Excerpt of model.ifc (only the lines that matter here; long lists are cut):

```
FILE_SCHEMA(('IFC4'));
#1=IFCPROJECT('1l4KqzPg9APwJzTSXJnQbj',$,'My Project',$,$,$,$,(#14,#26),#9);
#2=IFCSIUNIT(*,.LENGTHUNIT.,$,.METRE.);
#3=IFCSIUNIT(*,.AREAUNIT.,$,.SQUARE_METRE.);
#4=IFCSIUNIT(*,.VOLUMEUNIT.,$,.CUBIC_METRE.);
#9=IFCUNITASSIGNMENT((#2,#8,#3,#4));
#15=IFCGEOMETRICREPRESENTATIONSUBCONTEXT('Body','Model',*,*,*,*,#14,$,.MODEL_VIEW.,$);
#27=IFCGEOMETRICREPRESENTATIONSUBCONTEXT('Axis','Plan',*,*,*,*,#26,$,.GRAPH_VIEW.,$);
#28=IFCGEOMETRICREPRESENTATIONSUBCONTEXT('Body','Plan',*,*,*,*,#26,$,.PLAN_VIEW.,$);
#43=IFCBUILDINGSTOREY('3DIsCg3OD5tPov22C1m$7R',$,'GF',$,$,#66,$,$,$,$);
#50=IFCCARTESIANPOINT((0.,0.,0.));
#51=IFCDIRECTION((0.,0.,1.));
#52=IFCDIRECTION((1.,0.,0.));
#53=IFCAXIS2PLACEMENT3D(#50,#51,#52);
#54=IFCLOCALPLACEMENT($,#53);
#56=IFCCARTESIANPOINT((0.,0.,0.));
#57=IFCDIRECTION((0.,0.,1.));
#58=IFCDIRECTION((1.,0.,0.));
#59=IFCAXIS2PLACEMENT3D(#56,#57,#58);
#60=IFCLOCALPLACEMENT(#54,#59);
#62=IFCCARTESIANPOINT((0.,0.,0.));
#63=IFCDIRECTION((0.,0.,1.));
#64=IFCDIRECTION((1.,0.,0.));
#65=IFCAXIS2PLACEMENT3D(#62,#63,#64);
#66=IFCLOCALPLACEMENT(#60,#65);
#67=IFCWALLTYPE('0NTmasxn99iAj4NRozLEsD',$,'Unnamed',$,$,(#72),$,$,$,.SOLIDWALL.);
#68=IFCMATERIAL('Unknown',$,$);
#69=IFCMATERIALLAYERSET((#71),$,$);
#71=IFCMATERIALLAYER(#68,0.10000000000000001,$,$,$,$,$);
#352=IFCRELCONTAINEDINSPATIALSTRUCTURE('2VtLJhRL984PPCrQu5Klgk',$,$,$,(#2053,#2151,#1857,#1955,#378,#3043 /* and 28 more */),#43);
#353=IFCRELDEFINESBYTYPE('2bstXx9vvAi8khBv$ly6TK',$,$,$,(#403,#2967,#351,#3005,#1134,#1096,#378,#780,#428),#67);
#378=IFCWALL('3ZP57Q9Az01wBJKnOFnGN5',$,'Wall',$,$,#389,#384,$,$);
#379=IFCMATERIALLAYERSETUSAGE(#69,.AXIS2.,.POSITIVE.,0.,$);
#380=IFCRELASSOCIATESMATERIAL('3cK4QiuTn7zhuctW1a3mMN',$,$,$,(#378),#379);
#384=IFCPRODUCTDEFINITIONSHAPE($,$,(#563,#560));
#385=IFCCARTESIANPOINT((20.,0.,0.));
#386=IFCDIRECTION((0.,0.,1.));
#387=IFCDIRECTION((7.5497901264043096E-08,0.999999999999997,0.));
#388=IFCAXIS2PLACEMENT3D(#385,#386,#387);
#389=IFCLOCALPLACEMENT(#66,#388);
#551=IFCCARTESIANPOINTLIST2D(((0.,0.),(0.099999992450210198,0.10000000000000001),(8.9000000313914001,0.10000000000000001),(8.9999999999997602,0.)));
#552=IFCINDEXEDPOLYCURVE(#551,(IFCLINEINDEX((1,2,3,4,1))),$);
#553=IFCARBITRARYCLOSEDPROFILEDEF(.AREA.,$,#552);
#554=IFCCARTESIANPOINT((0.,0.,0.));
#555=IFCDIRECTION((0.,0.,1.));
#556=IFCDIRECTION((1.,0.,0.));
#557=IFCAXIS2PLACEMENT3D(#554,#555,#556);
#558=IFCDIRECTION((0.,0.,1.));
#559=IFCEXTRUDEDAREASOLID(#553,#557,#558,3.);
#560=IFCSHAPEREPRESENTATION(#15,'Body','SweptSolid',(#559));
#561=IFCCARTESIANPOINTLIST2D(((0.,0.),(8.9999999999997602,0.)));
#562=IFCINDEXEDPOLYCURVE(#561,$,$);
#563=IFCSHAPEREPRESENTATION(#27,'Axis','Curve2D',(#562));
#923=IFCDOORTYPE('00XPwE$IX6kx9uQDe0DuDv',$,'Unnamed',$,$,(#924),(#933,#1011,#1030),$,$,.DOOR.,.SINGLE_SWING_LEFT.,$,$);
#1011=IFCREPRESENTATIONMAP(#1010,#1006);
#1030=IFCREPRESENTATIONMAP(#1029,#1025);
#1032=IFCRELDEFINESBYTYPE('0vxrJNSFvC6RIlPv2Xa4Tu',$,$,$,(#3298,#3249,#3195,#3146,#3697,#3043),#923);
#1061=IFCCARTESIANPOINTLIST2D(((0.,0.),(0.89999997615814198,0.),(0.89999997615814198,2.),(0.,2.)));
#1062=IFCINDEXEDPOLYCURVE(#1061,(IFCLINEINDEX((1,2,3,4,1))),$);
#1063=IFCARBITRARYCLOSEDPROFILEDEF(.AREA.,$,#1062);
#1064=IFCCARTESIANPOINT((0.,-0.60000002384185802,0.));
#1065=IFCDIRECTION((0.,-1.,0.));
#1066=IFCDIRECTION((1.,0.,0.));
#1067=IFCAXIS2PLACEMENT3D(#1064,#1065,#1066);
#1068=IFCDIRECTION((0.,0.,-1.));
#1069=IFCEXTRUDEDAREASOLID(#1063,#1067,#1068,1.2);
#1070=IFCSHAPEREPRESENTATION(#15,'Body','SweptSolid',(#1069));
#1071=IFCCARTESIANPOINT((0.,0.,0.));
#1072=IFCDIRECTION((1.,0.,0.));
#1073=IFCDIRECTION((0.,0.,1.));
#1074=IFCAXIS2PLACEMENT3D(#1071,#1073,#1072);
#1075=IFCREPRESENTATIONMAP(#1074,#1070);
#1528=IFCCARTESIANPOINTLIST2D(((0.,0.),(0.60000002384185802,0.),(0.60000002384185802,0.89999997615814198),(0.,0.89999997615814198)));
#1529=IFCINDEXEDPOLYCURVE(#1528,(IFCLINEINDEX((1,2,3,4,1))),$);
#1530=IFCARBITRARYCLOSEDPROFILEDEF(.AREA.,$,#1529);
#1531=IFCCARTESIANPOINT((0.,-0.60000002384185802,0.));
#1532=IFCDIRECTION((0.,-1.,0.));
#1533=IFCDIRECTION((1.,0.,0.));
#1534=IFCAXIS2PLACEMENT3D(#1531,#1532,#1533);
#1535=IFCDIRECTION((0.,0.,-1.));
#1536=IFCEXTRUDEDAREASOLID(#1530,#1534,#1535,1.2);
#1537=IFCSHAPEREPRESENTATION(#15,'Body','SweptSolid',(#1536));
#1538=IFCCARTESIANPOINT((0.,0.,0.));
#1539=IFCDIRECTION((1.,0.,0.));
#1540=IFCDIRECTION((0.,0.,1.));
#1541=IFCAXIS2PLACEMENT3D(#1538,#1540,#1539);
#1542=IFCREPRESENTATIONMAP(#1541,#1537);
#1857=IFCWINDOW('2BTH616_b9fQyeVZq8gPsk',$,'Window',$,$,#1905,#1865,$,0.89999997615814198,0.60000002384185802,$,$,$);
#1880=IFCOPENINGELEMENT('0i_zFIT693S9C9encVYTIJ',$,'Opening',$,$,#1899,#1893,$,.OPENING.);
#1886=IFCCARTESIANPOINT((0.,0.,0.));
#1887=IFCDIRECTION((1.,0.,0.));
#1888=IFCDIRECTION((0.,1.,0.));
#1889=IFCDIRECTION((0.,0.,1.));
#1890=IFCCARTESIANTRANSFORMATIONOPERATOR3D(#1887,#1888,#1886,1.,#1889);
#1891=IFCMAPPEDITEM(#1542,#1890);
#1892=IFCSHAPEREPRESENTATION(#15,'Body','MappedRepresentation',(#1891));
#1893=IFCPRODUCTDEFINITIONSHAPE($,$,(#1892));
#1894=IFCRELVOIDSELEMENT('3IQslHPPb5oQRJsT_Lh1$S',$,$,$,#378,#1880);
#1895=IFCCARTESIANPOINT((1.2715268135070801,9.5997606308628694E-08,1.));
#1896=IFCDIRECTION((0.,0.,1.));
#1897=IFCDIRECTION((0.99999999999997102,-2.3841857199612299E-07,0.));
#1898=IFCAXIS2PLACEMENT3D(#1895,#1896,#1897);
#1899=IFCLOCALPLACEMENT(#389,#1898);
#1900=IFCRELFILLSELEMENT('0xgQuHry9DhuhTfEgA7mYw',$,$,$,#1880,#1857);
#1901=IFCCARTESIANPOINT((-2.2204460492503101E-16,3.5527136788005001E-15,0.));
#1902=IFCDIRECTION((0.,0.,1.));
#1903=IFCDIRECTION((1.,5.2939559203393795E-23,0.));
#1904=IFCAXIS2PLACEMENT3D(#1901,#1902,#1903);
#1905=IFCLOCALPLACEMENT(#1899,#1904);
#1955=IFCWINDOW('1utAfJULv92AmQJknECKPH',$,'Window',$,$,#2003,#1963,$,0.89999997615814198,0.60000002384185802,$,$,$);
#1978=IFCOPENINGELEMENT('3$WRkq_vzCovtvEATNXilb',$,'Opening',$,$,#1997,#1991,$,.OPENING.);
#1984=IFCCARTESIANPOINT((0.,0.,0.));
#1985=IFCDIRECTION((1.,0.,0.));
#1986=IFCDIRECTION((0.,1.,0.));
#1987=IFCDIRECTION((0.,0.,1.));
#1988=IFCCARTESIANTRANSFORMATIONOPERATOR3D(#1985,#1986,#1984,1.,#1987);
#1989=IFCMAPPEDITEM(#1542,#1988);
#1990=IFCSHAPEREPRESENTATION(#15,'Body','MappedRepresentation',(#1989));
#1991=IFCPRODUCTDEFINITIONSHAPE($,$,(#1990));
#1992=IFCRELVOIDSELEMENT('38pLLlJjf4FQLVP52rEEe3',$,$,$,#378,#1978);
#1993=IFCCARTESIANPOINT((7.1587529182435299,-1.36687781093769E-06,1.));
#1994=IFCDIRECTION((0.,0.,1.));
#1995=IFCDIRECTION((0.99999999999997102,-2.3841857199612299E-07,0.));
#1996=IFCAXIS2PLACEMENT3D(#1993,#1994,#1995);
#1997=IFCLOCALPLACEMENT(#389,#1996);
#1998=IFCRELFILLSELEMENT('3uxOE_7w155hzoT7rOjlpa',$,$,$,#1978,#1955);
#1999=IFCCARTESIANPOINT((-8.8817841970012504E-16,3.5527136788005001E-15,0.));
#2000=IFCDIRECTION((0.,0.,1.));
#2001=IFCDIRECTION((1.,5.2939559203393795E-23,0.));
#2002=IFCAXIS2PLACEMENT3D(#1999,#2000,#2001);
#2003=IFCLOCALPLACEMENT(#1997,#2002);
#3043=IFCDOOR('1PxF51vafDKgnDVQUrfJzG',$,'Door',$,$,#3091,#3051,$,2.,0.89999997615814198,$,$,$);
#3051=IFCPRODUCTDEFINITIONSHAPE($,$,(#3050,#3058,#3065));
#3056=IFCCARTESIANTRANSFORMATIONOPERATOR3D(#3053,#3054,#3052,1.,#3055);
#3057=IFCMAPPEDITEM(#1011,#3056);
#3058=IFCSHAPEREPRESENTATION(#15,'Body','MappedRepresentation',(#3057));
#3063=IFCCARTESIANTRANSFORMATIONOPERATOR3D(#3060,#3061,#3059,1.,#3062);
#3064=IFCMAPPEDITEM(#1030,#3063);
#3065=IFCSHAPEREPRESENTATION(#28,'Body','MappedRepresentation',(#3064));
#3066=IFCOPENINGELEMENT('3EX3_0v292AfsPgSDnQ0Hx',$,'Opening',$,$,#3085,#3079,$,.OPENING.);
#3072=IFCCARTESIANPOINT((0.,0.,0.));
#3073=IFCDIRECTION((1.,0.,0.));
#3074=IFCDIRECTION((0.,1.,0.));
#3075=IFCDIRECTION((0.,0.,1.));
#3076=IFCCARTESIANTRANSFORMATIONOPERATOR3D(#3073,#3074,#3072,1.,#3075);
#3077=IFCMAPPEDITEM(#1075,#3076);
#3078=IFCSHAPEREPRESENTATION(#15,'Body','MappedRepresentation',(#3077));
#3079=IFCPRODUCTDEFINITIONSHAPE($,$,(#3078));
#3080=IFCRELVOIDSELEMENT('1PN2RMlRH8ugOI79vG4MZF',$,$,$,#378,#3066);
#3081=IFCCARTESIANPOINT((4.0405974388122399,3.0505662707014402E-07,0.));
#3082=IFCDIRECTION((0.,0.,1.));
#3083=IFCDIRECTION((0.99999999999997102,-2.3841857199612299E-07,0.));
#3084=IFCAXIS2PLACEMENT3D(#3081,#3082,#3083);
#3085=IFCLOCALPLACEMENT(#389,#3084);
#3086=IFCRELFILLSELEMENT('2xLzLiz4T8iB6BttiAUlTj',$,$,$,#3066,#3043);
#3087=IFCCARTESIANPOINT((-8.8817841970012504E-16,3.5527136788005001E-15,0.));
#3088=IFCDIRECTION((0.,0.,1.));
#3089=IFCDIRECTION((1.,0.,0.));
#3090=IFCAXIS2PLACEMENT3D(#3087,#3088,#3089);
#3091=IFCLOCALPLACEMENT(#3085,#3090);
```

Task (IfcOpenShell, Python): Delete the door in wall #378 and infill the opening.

```python
import ifcopenshell
import ifcopenshell.api.feature
import ifcopenshell.api.root
import ifcopenshell.geom
import ifcopenshell.util.shape

model = ifcopenshell.open("model.ifc")
settings = ifcopenshell.geom.settings()


def volume(element):
    """Net volume in cubic metres, openings subtracted."""
    shape = ifcopenshell.geom.create_shape(settings, element)
    return ifcopenshell.util.shape.get_volume(shape.geometry)


door = model.by_id(3043)
opening = door.FillsVoids[0].RelatingOpeningElement
wall = opening.VoidsElements[0].RelatingBuildingElement
before = volume(wall)

ifcopenshell.api.root.remove_product(model, product=door)
ifcopenshell.api.feature.remove_feature(model, feature=opening)

after = volume(wall)

print(f"wall volume {before:.3f} -> {after:.3f} m3")

model.write("model_edited.ifc")
```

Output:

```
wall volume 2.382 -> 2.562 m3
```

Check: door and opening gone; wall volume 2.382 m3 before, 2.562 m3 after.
